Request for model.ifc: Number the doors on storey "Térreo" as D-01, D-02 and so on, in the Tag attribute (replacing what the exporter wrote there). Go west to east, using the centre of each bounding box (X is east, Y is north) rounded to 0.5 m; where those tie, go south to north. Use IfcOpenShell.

First a look at what the model holds.

```python
import ifcopenshell
import ifcopenshell.util.element
import ifcopenshell.util.placement

model = ifcopenshell.open("model.ifc")
print(model.schema)
storey = next(s for s in model.by_type("IfcBuildingStorey") if s.Name == "Térreo")
doors = [e for e in ifcopenshell.util.element.get_decomposition(storey) if e.is_a("IfcDoor")]
for e in sorted(doors, key=lambda e: e.id()):
    origin = ifcopenshell.util.placement.get_local_placement(e.ObjectPlacement)[:3, 3]
    print(e.id(), e.Tag, e.Name, origin.round(2) + 0.0, sep=" | ")
```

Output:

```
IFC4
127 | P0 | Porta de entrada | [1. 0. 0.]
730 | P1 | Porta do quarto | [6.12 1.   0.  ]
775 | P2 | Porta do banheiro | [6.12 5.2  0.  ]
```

```python
import ifcopenshell
import ifcopenshell.geom
import ifcopenshell.util.element
import ifcopenshell.util.shape

model = ifcopenshell.open("model.ifc")
settings = ifcopenshell.geom.settings()
settings.set("use-world-coords", True)


def centre(element):
    shape = ifcopenshell.geom.create_shape(settings, element)
    return ifcopenshell.util.shape.get_bbox_centroid(shape.geometry)


storey = next(s for s in model.by_type("IfcBuildingStorey") if s.Name == "Térreo")
doors = [e for e in ifcopenshell.util.element.get_decomposition(storey) if e.is_a("IfcDoor")]

# Insertion points can sit at a corner or the storey origin, so sort by the geometry (in metres).
centres = {e: centre(e) for e in doors}
doors.sort(key=lambda e: (round(centres[e][0] / 0.5), centres[e][1]))

for i, e in enumerate(doors, start=1):
    number = f"D-{i:02d}"
    e.Tag = number
    print(e.id(), number)

model.write("model-out.ifc")
```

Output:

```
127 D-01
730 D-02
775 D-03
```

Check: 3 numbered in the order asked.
